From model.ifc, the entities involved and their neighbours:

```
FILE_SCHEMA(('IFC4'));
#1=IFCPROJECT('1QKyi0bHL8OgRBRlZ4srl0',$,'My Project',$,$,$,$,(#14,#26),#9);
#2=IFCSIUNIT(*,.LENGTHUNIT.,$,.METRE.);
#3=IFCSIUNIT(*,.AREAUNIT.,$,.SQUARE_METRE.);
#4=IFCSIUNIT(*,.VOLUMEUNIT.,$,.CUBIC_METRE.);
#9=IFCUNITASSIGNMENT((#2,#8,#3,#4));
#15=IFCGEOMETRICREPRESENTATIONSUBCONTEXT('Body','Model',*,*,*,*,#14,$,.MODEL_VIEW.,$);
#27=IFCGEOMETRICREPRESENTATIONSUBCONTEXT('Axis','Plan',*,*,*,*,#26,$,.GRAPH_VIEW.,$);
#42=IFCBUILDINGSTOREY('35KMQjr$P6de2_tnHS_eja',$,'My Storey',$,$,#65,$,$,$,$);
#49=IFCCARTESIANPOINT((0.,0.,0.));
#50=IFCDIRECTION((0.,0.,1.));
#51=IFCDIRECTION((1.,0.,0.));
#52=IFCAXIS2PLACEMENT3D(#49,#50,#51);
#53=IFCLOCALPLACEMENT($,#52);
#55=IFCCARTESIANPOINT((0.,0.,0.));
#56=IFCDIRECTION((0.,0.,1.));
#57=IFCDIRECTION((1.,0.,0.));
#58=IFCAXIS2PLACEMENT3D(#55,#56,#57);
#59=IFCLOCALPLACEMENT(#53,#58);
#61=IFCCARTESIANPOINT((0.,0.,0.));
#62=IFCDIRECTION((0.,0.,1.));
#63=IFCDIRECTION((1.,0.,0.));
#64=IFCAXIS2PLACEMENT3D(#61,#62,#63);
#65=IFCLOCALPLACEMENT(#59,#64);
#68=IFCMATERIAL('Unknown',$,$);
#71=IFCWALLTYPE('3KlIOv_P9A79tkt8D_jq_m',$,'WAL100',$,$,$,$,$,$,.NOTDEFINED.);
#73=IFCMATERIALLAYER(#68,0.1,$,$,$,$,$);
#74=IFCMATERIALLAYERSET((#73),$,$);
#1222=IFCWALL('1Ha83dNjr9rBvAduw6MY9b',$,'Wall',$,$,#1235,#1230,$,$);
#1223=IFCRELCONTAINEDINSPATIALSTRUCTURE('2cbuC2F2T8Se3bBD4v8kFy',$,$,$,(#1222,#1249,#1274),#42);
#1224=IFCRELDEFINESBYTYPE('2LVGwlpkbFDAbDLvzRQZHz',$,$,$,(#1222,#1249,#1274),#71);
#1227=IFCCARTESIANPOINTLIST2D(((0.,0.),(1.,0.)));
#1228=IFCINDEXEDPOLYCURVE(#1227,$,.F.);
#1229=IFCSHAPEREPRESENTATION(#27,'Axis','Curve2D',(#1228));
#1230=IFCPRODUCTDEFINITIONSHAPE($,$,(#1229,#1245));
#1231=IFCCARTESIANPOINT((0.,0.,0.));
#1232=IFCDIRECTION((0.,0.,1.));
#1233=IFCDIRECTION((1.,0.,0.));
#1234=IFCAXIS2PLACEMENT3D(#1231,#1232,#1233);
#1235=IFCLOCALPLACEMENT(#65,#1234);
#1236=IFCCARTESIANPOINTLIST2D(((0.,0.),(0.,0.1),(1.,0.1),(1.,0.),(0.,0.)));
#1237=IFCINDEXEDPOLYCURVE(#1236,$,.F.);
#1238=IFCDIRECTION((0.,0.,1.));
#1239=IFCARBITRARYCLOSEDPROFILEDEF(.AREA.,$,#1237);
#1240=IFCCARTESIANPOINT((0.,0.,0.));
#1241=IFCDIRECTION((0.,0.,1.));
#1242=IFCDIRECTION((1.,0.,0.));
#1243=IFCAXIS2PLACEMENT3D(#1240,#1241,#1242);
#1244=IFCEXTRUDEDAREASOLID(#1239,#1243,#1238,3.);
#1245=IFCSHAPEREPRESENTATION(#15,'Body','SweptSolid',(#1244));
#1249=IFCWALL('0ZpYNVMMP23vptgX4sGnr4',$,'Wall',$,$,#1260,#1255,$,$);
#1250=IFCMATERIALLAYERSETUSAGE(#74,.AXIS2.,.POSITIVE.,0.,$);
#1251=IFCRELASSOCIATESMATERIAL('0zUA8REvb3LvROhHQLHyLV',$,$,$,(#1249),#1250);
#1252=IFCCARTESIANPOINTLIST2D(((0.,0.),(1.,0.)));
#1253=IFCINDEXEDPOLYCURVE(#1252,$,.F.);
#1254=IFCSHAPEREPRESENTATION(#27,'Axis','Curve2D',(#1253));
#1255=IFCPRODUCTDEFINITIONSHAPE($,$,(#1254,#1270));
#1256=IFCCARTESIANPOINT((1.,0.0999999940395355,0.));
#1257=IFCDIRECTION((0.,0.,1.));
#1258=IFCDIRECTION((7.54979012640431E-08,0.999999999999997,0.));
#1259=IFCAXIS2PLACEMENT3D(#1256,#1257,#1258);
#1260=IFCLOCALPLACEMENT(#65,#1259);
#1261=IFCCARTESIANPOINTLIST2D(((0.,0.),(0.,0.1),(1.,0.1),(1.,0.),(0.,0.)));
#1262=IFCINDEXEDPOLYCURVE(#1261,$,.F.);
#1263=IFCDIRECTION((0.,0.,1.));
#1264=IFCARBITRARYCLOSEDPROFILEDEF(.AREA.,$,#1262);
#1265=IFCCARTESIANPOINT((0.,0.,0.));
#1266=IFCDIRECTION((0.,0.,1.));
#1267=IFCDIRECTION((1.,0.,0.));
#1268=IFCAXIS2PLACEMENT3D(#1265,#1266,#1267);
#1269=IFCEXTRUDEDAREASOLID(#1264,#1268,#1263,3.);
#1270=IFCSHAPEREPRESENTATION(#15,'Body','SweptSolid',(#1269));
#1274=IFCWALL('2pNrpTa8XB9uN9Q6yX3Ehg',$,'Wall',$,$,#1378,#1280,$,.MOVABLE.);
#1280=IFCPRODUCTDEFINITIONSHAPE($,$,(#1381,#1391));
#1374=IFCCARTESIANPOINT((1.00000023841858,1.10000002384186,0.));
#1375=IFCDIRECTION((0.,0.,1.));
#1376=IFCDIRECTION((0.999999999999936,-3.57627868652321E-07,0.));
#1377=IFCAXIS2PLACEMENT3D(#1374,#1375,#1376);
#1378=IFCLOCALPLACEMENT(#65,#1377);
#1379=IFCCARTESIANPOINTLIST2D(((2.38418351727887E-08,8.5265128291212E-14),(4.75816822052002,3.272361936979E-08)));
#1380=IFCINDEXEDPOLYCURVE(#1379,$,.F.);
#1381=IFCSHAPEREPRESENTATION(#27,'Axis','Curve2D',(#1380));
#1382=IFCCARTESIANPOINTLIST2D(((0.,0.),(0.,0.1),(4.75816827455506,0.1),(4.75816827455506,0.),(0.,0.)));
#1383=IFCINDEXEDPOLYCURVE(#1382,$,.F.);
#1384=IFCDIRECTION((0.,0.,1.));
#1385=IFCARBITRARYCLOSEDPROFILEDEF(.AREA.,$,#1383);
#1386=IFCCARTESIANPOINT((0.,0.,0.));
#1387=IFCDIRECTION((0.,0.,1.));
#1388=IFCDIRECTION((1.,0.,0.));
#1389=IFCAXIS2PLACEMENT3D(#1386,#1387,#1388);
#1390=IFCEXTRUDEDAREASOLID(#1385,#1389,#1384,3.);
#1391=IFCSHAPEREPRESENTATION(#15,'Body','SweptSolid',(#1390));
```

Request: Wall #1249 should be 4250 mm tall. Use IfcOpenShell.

```python
import ifcopenshell
import ifcopenshell.geom
import ifcopenshell.util.representation
import ifcopenshell.util.shape

model = ifcopenshell.open("model.ifc")
settings = ifcopenshell.geom.settings()


def volume(element):
    """Net volume in cubic metres, openings subtracted."""
    shape = ifcopenshell.geom.create_shape(settings, element)
    return ifcopenshell.util.shape.get_volume(shape.geometry)


wall = model.by_id(1249)
before = volume(wall)

body = ifcopenshell.util.representation.get_representation(wall, "Model", "Body")
solid = body.Items[0]
old_height = solid.Depth
solid.Depth = 4.25
after = volume(wall)

print(f"height {old_height:g} -> {solid.Depth:g}, volume {before:.3f} -> {after:.3f} m3")

model.write("model_rev.ifc")
```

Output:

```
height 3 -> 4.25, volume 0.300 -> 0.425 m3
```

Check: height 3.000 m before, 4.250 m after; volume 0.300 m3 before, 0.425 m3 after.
